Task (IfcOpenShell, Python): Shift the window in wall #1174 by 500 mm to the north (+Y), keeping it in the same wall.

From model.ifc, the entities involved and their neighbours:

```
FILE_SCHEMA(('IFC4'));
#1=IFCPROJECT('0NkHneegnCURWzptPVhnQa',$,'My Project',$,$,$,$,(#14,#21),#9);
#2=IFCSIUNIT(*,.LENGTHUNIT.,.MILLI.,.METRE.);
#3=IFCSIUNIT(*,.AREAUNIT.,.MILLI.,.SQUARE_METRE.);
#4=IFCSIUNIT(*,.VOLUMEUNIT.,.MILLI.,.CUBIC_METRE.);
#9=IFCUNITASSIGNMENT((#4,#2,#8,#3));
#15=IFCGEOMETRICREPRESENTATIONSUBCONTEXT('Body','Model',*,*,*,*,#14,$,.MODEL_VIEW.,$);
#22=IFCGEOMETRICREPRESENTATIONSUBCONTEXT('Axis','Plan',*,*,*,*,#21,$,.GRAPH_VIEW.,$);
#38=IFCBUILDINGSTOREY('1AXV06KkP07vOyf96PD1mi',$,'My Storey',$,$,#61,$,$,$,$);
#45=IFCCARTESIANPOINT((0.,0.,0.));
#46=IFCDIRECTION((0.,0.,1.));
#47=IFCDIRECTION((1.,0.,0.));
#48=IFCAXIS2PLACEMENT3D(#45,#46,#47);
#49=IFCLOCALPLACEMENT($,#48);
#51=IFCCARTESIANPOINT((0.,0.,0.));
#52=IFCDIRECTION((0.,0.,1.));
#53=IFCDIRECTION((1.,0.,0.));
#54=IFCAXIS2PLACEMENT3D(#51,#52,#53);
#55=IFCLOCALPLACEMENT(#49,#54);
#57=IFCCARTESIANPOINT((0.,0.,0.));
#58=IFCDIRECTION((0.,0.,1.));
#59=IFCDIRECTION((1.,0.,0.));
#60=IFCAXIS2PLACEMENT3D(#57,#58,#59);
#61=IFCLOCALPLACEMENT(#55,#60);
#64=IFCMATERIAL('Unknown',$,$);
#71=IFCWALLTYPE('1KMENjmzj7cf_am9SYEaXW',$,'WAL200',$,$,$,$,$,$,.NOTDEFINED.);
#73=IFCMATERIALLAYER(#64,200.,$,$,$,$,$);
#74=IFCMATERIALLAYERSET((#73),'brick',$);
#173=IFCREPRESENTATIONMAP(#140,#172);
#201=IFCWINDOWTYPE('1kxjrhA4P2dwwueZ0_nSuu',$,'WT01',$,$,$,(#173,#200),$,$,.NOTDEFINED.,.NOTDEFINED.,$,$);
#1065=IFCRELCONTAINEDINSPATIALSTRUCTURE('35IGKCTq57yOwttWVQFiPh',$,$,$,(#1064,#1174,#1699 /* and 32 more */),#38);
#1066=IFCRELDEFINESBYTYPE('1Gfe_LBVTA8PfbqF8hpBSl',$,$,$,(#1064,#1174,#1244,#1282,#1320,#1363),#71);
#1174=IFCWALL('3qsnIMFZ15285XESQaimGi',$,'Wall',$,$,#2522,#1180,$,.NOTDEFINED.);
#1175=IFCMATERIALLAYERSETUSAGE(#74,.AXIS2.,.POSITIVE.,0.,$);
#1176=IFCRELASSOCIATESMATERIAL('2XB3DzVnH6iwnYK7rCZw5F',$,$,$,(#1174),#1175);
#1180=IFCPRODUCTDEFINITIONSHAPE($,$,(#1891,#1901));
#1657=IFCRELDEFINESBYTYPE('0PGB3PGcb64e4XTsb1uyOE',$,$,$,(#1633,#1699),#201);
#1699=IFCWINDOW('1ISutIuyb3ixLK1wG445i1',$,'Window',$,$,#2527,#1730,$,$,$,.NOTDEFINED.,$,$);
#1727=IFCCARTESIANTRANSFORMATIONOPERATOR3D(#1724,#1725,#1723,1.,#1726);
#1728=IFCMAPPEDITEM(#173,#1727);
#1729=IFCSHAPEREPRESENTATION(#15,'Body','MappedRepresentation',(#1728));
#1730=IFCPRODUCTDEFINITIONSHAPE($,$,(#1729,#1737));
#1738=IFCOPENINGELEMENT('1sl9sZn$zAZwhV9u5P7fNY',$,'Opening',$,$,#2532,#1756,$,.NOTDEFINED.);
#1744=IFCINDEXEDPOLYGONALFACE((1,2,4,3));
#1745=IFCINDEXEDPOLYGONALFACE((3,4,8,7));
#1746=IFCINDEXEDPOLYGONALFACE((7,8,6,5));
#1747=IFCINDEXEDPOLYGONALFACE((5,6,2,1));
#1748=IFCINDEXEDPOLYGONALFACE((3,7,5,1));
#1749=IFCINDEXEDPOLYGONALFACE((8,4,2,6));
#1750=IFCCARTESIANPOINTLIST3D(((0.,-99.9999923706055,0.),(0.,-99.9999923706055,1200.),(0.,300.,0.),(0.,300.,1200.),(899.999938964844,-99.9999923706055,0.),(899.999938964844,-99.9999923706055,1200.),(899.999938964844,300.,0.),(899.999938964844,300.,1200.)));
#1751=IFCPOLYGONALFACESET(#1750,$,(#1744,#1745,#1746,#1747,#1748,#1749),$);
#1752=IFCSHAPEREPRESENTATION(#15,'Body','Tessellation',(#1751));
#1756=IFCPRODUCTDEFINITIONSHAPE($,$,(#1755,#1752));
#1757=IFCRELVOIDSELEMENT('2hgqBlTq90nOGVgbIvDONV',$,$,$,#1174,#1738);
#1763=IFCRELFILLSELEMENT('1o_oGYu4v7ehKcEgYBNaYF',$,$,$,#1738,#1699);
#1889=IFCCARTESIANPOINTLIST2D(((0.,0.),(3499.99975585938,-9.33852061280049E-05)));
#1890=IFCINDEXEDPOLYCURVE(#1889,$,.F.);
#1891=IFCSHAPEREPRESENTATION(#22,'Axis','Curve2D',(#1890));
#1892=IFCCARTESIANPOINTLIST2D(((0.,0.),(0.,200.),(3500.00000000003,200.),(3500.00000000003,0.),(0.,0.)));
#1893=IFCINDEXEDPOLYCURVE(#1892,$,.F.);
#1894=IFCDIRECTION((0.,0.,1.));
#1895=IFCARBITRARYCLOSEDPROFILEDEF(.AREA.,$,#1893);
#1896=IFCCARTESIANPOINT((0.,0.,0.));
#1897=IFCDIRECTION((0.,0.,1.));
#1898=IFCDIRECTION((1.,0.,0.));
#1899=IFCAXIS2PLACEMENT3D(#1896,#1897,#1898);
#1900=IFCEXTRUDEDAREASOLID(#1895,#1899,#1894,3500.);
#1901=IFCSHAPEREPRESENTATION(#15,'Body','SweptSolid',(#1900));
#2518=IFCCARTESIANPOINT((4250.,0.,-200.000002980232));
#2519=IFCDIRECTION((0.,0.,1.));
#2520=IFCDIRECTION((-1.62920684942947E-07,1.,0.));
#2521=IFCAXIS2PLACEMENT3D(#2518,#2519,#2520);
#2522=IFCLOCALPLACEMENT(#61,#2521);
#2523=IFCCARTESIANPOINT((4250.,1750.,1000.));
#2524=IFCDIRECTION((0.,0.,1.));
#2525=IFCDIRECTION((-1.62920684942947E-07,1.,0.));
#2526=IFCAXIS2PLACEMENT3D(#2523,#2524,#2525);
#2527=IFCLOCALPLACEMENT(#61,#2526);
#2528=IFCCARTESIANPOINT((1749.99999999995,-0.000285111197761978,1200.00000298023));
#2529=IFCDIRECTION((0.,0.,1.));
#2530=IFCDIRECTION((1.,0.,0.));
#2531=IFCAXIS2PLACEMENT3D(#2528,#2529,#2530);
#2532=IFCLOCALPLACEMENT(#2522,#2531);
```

```python
import ifcopenshell
import ifcopenshell.api.geometry
import ifcopenshell.util.placement
import ifcopenshell.util.unit

model = ifcopenshell.open("model.ifc")
unit_scale = ifcopenshell.util.unit.calculate_unit_scale(model)

window = model.by_id(1699)
opening = window.FillsVoids[0].RelatingOpeningElement
wall = opening.VoidsElements[0].RelatingBuildingElement

wall_matrix = ifcopenshell.util.placement.get_local_placement(wall.ObjectPlacement)
shift = wall_matrix[:3, 0] * 0.5 / unit_scale
before = ifcopenshell.util.placement.get_local_placement(window.ObjectPlacement)[:3, 3].copy()

# The window is not placed relative to its opening, so move both.
for product in (opening, window):
    matrix = ifcopenshell.util.placement.get_local_placement(product.ObjectPlacement)
    matrix[:3, 3] += shift
    ifcopenshell.api.geometry.edit_object_placement(model, product=product, matrix=matrix, is_si=False)

after = ifcopenshell.util.placement.get_local_placement(window.ObjectPlacement)[:3, 3]
print("window moved by", (after - before).round(3) + 0.0)

model.write("model_updated.ifc")
```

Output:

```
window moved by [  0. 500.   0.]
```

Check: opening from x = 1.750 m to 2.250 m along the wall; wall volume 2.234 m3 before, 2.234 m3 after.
